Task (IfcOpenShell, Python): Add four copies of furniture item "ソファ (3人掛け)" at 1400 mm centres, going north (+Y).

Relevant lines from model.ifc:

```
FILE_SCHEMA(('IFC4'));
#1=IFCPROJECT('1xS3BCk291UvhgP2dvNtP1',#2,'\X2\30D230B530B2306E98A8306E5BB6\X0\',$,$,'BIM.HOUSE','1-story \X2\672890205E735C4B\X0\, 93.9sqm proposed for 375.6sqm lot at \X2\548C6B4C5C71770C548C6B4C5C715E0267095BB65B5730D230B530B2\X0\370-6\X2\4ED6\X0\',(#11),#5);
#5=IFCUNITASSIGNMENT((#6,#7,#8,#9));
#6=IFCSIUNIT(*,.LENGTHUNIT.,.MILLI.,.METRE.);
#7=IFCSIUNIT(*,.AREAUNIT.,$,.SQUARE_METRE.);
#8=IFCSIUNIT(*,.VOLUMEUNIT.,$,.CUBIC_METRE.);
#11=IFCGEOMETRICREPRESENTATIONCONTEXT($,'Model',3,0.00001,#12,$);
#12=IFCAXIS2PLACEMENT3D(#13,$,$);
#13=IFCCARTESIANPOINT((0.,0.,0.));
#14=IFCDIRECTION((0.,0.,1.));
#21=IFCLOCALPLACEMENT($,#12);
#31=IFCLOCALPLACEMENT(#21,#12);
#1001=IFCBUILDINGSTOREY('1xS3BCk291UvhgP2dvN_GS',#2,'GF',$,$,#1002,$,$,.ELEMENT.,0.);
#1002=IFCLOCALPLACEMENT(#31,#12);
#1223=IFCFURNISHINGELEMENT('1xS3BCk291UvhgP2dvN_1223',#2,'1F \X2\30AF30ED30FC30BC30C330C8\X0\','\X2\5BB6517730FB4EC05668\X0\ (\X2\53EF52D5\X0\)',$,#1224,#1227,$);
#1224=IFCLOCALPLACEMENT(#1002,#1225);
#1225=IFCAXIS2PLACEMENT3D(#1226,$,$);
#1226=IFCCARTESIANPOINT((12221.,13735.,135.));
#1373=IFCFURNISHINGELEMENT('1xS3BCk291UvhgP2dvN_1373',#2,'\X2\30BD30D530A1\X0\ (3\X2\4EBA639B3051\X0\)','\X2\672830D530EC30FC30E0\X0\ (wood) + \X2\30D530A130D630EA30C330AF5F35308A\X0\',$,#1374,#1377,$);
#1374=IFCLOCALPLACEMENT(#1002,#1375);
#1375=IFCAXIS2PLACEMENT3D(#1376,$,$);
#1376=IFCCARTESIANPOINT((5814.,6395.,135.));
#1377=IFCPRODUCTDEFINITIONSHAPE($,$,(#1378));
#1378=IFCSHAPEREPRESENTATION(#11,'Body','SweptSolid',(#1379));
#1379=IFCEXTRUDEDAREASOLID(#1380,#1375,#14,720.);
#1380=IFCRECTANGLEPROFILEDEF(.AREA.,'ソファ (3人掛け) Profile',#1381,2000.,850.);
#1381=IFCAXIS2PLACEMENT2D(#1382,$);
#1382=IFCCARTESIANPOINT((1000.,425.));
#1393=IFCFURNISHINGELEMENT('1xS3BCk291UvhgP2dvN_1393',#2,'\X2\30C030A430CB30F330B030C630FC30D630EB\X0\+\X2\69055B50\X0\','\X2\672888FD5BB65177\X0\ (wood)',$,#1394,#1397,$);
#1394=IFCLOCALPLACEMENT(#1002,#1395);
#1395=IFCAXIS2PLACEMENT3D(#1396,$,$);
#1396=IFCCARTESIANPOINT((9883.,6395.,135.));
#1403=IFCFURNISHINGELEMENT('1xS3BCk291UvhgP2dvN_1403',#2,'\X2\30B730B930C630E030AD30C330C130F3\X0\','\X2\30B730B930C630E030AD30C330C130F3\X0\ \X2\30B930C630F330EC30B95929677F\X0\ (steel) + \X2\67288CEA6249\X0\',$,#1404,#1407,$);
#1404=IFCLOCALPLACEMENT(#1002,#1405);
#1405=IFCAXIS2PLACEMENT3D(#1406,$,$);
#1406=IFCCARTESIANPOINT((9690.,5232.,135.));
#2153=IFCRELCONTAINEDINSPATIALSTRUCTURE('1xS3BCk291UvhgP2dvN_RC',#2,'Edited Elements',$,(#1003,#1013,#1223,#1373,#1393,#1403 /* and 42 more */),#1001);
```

```python
import numpy as np
import ifcopenshell
import ifcopenshell.api.geometry
import ifcopenshell.api.root
import ifcopenshell.util.element
import ifcopenshell.util.placement
import ifcopenshell.util.unit

model = ifcopenshell.open("model.ifc")
unit_scale = ifcopenshell.util.unit.calculate_unit_scale(model)


def reuse_history(source, copy):
    """copy_class also copies each property set's owner history, people and application; keep the originals."""
    for rel in copy.IsDefinedBy:
        if rel.is_a("IfcRelDefinesByProperties") and (history := rel.RelatingPropertyDefinition.OwnerHistory):
            rel.RelatingPropertyDefinition.OwnerHistory = source.OwnerHistory
            ifcopenshell.util.element.remove_deep2(model, history)


source = model.by_guid("1xS3BCk291UvhgP2dvN_1373")
base = ifcopenshell.util.placement.get_local_placement(source.ObjectPlacement)
step = np.array([0.0, 1.0, 0.0]) * 1.4 / unit_scale

for i in range(1, 5):
    copy = ifcopenshell.api.root.copy_class(model, product=source)
    copy.Representation = ifcopenshell.util.element.copy_deep(
        model, source.Representation, exclude=["IfcGeometricRepresentationContext", "IfcRepresentationMap"]
    )
    reuse_history(source, copy)
    matrix = base.copy()
    matrix[:3, 3] += i * step
    print("added at", matrix[:3, 3].round(3) + 0.0)
    ifcopenshell.api.geometry.edit_object_placement(model, product=copy, matrix=matrix, is_si=False)

model.write("model_edited.ifc")
```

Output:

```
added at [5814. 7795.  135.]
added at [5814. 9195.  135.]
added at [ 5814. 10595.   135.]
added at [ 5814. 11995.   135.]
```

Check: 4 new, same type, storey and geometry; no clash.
